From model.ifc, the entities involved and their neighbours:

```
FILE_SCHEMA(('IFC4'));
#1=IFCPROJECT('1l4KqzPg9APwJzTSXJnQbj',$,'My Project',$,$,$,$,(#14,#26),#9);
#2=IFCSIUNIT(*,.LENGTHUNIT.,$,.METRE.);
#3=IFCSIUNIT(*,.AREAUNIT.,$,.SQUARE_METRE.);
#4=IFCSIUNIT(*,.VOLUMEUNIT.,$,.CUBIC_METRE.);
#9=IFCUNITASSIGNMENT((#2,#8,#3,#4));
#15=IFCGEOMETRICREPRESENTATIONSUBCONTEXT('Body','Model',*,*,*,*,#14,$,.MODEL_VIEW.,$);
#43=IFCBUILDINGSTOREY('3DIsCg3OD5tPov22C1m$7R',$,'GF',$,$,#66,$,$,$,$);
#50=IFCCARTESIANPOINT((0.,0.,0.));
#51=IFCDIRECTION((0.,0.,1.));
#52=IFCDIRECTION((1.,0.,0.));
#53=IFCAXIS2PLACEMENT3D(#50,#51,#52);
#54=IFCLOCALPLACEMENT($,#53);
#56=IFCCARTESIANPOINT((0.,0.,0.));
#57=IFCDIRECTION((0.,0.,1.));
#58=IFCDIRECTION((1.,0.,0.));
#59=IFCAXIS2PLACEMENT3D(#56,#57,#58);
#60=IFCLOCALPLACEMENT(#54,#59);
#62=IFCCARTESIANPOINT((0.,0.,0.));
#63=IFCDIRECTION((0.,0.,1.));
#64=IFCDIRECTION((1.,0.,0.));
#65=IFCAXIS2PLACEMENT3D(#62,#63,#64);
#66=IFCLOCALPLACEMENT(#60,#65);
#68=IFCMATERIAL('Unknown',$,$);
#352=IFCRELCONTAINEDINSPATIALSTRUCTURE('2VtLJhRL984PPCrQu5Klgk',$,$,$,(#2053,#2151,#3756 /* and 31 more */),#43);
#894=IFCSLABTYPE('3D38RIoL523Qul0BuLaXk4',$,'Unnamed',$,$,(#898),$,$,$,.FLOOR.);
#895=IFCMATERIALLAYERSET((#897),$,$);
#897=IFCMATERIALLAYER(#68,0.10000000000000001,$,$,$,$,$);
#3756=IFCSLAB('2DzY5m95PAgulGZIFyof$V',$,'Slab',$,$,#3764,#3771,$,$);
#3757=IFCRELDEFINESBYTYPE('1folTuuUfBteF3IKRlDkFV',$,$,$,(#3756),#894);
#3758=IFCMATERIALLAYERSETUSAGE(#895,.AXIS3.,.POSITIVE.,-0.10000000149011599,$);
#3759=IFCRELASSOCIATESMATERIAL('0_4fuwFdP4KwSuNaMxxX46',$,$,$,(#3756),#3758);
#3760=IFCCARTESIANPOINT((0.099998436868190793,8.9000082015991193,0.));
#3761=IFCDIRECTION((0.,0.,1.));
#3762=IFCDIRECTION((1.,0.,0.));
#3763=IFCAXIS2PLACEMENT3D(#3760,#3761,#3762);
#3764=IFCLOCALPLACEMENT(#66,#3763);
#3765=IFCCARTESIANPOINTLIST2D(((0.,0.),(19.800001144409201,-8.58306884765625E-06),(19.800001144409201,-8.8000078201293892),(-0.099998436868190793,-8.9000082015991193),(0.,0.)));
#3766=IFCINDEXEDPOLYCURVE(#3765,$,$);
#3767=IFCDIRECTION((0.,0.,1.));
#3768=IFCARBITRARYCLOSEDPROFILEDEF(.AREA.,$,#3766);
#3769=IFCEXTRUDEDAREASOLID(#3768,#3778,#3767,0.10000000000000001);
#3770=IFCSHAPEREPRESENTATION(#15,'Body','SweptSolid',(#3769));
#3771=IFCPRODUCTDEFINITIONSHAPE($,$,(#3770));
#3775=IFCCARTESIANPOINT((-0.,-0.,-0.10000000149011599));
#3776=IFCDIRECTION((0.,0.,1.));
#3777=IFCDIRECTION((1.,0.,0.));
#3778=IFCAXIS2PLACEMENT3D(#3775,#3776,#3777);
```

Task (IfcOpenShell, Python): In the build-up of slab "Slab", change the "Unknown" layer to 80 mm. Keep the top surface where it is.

```python
import ifcopenshell
import ifcopenshell.util.element
import ifcopenshell.util.representation
import ifcopenshell.util.unit

model = ifcopenshell.open("model.ifc")
unit_scale = ifcopenshell.util.unit.calculate_unit_scale(model)

layer_set = model.by_id(895)
layer = next(l for l in layer_set.MaterialLayers if l.Material and l.Material.Name == "Unknown")
change = 0.08 / unit_scale - layer.LayerThickness
layer.LayerThickness += change

# Geometry does not follow the layer set by itself.
slabs = [e for e in ifcopenshell.util.element.get_elements_by_material(model, layer_set) if e.is_a("IfcSlab")]
for slab in sorted(slabs, key=lambda e: e.id()):
    body = ifcopenshell.util.representation.get_representation(slab, "Model", "Body")
    solid = body.Items[0]
    old_depth = solid.Depth
    solid.Depth += change
    # Extruded upwards: lower the start of the extrusion so the top stays.
    x, y, z = solid.Position.Location.Coordinates
    solid.Position.Location = model.createIfcCartesianPoint((x, y, z - change))
    print(slab.id(), f"{old_depth:g} -> {solid.Depth:g}")

# The layers are counted up from the underside, which has moved.
for usage in {ifcopenshell.util.element.get_material(slab) for slab in slabs}:
    usage.OffsetFromReferenceLine -= change

model.write("model-out.ifc")
```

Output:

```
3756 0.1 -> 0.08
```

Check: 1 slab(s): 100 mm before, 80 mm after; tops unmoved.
